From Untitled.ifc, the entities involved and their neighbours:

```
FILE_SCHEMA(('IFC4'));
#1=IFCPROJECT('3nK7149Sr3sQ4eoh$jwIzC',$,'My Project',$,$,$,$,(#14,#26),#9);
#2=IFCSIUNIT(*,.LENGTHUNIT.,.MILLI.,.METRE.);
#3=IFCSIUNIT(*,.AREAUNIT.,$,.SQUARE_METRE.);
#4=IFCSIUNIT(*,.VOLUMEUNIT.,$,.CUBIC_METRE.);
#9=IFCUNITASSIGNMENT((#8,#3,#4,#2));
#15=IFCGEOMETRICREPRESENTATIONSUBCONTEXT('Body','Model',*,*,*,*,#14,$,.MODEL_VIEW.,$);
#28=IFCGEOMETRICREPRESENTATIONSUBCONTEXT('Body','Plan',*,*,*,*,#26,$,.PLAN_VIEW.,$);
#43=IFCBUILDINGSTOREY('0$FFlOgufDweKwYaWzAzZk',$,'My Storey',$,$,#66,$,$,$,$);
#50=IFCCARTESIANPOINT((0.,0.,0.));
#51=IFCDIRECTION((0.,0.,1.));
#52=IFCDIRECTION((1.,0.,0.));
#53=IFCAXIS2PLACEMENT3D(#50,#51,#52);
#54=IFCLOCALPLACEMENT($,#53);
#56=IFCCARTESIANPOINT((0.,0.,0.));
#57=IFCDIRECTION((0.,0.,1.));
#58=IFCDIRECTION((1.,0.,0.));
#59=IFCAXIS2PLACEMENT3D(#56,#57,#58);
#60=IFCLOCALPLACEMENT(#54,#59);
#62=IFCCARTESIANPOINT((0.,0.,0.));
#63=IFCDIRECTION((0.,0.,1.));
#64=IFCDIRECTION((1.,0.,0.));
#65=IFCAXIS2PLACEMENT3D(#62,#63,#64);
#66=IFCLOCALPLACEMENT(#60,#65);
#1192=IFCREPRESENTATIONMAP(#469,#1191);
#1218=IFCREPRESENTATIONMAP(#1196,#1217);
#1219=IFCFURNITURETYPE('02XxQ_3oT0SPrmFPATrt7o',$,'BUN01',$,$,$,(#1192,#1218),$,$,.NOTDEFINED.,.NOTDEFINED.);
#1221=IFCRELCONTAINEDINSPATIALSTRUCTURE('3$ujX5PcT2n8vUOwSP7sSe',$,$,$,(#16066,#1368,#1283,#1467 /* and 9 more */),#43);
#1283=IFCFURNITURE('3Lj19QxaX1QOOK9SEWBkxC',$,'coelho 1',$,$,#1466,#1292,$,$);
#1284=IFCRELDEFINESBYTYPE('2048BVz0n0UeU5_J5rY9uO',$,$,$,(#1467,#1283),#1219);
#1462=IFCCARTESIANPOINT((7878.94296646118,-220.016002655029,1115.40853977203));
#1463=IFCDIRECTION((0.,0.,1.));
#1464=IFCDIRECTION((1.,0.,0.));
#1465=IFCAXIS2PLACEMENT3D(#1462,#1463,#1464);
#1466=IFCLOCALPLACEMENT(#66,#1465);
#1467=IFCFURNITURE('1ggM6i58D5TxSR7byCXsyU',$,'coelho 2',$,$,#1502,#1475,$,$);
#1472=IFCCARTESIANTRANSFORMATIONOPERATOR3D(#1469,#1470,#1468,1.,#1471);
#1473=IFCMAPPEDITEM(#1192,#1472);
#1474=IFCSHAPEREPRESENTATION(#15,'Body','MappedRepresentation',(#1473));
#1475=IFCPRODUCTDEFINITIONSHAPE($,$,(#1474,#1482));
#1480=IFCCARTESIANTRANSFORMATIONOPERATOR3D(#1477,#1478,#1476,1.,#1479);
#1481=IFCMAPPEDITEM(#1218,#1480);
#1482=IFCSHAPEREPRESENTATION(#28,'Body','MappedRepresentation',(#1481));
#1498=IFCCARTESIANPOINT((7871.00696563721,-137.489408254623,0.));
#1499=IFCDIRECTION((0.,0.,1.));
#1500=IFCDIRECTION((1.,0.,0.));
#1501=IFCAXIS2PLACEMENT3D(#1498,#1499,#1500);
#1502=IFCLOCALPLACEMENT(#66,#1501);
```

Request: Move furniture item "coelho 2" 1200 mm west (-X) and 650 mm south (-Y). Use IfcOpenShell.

```python
import ifcopenshell
import ifcopenshell.api.geometry
import ifcopenshell.util.placement

model = ifcopenshell.open("Untitled.ifc")

item = model.by_guid("1ggM6i58D5TxSR7byCXsyU")
matrix = ifcopenshell.util.placement.get_local_placement(item.ObjectPlacement)
matrix[0, 3] -= 1200.0
matrix[1, 3] -= 650.0
ifcopenshell.api.geometry.edit_object_placement(model, product=item, matrix=matrix, is_si=False)

print(ifcopenshell.util.placement.get_local_placement(item.ObjectPlacement).round(3) + 0.0)

model.write("Untitled_updated.ifc")
```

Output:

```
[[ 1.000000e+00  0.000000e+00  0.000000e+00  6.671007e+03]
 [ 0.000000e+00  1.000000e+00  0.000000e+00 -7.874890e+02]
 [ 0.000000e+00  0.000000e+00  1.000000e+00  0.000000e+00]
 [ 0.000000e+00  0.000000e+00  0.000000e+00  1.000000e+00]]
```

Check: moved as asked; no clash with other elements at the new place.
